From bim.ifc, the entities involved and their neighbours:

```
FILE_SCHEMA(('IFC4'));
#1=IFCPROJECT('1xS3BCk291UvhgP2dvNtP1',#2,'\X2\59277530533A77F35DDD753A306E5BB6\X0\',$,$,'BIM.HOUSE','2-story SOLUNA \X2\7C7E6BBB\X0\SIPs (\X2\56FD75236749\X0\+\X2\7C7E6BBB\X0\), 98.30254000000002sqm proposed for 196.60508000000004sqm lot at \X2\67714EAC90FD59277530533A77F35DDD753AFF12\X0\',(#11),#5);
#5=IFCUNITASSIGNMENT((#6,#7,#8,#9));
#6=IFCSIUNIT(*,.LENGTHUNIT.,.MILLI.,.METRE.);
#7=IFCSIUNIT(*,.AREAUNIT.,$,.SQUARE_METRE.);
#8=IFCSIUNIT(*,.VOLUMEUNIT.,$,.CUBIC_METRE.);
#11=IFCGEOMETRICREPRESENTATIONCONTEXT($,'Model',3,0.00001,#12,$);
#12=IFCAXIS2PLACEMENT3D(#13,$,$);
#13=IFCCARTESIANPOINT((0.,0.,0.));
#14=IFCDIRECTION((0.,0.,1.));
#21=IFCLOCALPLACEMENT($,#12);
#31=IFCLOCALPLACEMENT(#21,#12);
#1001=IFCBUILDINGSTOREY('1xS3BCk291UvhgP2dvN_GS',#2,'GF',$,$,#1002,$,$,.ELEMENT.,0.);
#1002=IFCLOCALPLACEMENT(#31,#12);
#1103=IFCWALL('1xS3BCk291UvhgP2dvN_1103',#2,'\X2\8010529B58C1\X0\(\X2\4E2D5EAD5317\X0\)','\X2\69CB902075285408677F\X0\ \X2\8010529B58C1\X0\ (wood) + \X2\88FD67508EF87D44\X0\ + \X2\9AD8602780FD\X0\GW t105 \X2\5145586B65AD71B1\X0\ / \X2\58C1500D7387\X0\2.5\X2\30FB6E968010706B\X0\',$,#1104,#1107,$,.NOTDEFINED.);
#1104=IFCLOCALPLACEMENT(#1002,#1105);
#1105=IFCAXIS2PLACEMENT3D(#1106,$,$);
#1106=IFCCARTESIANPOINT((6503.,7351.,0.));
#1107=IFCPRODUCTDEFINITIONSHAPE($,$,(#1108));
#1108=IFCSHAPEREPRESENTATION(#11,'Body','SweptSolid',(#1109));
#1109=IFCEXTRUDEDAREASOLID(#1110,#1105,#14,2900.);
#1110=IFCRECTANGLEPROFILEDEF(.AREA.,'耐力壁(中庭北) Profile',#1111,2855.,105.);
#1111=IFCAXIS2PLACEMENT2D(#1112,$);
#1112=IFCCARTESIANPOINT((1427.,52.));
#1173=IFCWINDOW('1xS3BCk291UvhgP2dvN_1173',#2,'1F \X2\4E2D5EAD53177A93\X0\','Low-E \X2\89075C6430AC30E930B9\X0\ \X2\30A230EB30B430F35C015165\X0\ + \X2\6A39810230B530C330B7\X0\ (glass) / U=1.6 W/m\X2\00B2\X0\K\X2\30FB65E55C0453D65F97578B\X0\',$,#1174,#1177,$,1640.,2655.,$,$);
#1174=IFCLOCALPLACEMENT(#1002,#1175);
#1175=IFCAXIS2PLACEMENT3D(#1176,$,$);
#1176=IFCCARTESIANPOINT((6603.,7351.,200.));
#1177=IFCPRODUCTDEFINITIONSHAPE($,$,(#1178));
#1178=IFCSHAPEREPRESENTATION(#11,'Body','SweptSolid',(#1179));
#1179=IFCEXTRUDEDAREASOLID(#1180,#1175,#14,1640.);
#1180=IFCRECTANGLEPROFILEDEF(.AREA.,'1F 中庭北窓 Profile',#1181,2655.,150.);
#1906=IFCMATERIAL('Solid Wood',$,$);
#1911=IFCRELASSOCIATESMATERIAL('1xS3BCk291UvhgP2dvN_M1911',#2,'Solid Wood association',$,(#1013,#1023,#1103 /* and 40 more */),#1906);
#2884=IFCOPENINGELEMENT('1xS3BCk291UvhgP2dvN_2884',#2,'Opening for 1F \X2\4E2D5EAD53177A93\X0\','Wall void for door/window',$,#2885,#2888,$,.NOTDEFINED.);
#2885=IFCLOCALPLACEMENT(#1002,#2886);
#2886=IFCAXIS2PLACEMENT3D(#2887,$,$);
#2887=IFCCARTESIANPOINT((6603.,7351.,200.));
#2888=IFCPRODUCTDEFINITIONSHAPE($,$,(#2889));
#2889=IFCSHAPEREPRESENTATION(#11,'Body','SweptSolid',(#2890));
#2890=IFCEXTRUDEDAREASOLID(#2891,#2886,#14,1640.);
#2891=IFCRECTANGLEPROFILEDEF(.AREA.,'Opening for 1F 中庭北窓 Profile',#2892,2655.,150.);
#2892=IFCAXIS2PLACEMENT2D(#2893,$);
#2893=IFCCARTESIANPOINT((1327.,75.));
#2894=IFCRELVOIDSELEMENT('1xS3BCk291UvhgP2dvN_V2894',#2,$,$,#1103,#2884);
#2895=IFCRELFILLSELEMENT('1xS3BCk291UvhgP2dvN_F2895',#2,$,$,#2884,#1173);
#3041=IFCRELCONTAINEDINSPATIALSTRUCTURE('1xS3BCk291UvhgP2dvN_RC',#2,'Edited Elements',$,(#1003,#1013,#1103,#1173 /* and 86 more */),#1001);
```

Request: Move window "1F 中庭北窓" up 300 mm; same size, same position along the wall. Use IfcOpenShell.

```python
import numpy as np
import ifcopenshell
import ifcopenshell.api.geometry
import ifcopenshell.util.placement
import ifcopenshell.util.unit

model = ifcopenshell.open("bim.ifc")
unit_scale = ifcopenshell.util.unit.calculate_unit_scale(model)

window = model.by_guid("1xS3BCk291UvhgP2dvN_1173")
opening = window.FillsVoids[0].RelatingOpeningElement
dz = 0.3 / unit_scale

shift = np.array([0.0, 0.0, dz])
# The window is not placed relative to its opening, so move both.
for product in (opening, window):
    matrix = ifcopenshell.util.placement.get_local_placement(product.ObjectPlacement)
    matrix[:3, 3] += shift
    ifcopenshell.api.geometry.edit_object_placement(model, product=product, matrix=matrix, is_si=False)

print(f"moved by {dz * unit_scale:+.3f} m")

model.write("bim_rev.ifc")
```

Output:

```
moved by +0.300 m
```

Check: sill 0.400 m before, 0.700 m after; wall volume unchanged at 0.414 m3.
